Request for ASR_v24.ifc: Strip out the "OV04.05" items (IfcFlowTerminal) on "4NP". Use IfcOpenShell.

First a look at what the model holds.

```python
import ifcopenshell
import ifcopenshell.util.element

model = ifcopenshell.open("ASR_v24.ifc")
print(model.schema)
storey = next(s for s in model.by_type("IfcBuildingStorey") if s.Name == "4NP")
terminals = [e for e in ifcopenshell.util.element.get_decomposition(storey) if e.is_a("IfcFlowTerminal")]
seen = {}
for e in terminals:
    element_type = ifcopenshell.util.element.get_type(e)
    name = element_type.Name if element_type not in (None, e) else None
    seen[name] = seen.get(name, 0) + 1
for name, count in sorted(seen.items(), key=str):
    print(count, "x", name)
```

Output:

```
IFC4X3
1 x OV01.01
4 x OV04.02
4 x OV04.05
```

```python
import ifcopenshell
import ifcopenshell.api.root
import ifcopenshell.util.element

model = ifcopenshell.open("ASR_v24.ifc")

storey = next(s for s in model.by_type("IfcBuildingStorey") if s.Name == "4NP")
terminals = [e for e in ifcopenshell.util.element.get_decomposition(storey) if e.is_a("IfcFlowTerminal")]
targets = [e for e in terminals if (t := ifcopenshell.util.element.get_type(e)) not in (None, e) and t.Name == "OV04.05"]

for e in targets:
    ifcopenshell.api.root.remove_product(model, product=e)
print(len(targets), "removed")

model.write("ASR_v24_edited.ifc")
```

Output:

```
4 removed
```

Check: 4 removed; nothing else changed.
